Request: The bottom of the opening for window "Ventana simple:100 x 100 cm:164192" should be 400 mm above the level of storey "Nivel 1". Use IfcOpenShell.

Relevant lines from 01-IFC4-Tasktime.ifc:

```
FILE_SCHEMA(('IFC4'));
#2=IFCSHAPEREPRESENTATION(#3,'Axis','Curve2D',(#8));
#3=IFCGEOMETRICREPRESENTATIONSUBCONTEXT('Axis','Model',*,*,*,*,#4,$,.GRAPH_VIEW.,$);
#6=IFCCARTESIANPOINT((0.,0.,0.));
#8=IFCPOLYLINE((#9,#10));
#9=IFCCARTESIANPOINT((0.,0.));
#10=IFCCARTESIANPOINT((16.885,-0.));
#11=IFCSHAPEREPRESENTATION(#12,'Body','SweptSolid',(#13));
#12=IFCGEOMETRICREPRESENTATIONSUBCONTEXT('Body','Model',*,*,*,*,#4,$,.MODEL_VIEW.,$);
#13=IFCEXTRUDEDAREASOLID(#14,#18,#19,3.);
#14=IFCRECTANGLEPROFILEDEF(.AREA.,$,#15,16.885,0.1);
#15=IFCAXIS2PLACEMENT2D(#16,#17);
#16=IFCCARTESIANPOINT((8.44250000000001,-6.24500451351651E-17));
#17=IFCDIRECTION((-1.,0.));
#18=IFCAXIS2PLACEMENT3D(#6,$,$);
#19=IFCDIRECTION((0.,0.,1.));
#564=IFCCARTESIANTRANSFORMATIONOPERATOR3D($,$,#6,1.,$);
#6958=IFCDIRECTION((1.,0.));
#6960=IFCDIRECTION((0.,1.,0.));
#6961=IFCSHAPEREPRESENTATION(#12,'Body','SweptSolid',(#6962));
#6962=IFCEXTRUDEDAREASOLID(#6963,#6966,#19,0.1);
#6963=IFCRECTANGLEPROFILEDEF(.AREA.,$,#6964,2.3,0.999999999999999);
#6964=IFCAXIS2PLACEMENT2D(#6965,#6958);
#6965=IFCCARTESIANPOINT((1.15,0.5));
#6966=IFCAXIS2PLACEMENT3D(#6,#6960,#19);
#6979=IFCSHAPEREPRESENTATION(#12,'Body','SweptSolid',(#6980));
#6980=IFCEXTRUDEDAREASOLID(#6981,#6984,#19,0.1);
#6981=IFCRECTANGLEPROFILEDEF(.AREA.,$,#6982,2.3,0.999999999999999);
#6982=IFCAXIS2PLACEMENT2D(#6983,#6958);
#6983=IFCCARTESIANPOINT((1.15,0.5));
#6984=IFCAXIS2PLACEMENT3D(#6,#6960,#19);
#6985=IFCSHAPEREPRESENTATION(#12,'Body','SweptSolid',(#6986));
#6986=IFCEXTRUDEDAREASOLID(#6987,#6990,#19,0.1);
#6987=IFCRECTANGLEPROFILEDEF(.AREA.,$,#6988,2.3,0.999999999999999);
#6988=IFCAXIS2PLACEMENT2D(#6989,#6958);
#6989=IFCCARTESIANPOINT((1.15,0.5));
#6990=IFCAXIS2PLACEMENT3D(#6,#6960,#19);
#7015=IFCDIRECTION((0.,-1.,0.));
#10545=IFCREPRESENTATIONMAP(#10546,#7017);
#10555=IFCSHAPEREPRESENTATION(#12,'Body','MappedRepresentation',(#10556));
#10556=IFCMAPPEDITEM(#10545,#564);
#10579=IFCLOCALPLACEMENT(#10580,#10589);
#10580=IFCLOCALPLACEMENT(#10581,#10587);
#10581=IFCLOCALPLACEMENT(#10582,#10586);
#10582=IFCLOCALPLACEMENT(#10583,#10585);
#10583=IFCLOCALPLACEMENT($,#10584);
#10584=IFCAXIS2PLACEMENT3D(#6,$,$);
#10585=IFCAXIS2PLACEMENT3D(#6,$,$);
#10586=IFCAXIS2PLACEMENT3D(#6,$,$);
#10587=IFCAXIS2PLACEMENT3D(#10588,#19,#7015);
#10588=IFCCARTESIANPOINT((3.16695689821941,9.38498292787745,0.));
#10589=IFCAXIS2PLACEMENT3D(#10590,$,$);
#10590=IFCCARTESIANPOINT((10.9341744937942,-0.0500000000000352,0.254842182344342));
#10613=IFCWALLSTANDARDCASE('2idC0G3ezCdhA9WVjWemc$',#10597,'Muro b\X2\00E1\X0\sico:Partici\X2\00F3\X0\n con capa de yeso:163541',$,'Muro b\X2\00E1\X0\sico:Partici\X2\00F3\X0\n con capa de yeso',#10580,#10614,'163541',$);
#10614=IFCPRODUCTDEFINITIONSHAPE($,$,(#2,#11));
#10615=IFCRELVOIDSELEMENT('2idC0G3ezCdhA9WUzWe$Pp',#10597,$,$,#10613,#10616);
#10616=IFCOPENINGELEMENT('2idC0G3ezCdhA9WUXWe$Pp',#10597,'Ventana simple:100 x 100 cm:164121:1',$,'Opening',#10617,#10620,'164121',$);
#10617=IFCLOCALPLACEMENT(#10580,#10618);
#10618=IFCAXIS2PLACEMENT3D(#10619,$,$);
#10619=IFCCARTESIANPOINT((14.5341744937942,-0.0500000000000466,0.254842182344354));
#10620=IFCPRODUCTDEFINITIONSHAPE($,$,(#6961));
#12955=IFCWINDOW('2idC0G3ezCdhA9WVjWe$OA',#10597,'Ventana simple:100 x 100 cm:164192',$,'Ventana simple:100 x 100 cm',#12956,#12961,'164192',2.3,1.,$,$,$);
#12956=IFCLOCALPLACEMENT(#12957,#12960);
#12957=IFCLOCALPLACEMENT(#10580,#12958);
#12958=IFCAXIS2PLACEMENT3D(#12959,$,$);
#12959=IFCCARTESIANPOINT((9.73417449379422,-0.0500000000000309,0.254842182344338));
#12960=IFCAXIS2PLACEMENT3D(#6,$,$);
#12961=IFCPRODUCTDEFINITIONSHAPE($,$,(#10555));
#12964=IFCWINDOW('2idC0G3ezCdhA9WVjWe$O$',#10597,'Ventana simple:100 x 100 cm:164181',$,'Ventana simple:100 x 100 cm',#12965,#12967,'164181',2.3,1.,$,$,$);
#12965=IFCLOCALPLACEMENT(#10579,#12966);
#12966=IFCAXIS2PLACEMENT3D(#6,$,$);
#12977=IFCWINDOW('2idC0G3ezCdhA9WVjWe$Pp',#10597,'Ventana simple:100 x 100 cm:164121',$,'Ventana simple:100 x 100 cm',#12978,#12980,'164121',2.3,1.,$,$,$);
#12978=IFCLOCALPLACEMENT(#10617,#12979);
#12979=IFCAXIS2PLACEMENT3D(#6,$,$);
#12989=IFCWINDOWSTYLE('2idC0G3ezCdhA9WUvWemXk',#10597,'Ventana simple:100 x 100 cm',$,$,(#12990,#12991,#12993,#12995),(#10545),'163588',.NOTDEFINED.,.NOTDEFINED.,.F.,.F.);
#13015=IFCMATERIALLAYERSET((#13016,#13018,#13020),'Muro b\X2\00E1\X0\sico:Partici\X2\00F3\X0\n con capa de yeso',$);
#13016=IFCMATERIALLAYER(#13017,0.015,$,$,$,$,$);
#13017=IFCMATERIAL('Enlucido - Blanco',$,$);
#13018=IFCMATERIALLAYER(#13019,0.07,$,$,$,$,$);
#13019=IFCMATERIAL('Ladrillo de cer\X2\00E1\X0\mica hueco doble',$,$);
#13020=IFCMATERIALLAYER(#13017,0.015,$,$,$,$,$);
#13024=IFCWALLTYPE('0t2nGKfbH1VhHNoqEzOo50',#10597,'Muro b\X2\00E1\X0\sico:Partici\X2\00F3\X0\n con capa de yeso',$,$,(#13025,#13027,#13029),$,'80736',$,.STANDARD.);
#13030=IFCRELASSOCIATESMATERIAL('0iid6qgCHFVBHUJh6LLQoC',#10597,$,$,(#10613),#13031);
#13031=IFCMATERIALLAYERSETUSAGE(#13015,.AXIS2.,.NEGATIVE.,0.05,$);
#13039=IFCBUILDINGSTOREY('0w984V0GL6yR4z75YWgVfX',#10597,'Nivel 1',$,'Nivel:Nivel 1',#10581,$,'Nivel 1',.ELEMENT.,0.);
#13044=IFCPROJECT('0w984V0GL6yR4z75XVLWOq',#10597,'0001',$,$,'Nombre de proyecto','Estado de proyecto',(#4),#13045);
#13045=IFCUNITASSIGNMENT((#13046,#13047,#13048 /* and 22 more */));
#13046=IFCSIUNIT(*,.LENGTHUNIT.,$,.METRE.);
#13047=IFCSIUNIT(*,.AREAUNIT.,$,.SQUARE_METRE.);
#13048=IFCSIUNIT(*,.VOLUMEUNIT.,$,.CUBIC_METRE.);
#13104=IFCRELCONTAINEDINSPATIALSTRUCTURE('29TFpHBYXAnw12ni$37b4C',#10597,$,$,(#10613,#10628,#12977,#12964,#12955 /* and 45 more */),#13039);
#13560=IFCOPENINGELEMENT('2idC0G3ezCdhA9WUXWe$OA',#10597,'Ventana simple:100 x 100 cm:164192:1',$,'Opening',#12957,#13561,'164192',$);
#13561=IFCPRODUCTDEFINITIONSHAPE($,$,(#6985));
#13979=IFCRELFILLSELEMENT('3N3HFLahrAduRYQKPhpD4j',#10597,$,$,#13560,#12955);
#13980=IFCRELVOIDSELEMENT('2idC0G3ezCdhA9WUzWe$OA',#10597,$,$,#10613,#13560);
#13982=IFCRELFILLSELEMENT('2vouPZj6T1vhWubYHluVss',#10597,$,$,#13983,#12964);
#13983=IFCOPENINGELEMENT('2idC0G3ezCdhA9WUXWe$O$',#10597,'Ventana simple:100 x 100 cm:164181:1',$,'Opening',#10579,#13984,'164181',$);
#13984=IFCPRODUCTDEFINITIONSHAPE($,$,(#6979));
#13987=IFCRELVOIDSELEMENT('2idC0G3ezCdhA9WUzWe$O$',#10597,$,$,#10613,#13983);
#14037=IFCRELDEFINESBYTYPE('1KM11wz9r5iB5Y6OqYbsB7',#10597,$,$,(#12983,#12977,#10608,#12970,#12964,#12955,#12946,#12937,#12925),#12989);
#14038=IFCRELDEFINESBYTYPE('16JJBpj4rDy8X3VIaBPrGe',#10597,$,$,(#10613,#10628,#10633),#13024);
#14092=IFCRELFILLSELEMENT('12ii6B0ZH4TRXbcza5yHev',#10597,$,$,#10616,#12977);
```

```python
import numpy as np
import ifcopenshell
import ifcopenshell.api.geometry
import ifcopenshell.geom
import ifcopenshell.util.element
import ifcopenshell.util.placement
import ifcopenshell.util.shape
import ifcopenshell.util.unit

model = ifcopenshell.open("01-IFC4-Tasktime.ifc")
unit_scale = ifcopenshell.util.unit.calculate_unit_scale(model)

window = model.by_guid("2idC0G3ezCdhA9WVjWe$OA")
opening = window.FillsVoids[0].RelatingOpeningElement
storey = ifcopenshell.util.element.get_container(window, ifc_class="IfcBuildingStorey")
level = ifcopenshell.util.placement.get_local_placement(storey.ObjectPlacement)[2, 3]

# The opening's origin need not be at the sill, so measure its lowest point.
shape = ifcopenshell.geom.create_shape(ifcopenshell.geom.settings(), opening)
bottom = ifcopenshell.util.shape.get_shape_bottom_elevation(shape, shape.geometry) / unit_scale
dz = level + 0.4 - bottom

shift = np.array([0.0, 0.0, dz])
# The window is placed relative to its opening, so it follows when the opening moves.
matrix = ifcopenshell.util.placement.get_local_placement(opening.ObjectPlacement)
matrix[:3, 3] += shift
ifcopenshell.api.geometry.edit_object_placement(
    model, product=opening, matrix=matrix, is_si=False, should_transform_children=True
)

print(f"moved by {dz * unit_scale:+.3f} m")

model.write("01-IFC4-Tasktime_v2.ifc")
```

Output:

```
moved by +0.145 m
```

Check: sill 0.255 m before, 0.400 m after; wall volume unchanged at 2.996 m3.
